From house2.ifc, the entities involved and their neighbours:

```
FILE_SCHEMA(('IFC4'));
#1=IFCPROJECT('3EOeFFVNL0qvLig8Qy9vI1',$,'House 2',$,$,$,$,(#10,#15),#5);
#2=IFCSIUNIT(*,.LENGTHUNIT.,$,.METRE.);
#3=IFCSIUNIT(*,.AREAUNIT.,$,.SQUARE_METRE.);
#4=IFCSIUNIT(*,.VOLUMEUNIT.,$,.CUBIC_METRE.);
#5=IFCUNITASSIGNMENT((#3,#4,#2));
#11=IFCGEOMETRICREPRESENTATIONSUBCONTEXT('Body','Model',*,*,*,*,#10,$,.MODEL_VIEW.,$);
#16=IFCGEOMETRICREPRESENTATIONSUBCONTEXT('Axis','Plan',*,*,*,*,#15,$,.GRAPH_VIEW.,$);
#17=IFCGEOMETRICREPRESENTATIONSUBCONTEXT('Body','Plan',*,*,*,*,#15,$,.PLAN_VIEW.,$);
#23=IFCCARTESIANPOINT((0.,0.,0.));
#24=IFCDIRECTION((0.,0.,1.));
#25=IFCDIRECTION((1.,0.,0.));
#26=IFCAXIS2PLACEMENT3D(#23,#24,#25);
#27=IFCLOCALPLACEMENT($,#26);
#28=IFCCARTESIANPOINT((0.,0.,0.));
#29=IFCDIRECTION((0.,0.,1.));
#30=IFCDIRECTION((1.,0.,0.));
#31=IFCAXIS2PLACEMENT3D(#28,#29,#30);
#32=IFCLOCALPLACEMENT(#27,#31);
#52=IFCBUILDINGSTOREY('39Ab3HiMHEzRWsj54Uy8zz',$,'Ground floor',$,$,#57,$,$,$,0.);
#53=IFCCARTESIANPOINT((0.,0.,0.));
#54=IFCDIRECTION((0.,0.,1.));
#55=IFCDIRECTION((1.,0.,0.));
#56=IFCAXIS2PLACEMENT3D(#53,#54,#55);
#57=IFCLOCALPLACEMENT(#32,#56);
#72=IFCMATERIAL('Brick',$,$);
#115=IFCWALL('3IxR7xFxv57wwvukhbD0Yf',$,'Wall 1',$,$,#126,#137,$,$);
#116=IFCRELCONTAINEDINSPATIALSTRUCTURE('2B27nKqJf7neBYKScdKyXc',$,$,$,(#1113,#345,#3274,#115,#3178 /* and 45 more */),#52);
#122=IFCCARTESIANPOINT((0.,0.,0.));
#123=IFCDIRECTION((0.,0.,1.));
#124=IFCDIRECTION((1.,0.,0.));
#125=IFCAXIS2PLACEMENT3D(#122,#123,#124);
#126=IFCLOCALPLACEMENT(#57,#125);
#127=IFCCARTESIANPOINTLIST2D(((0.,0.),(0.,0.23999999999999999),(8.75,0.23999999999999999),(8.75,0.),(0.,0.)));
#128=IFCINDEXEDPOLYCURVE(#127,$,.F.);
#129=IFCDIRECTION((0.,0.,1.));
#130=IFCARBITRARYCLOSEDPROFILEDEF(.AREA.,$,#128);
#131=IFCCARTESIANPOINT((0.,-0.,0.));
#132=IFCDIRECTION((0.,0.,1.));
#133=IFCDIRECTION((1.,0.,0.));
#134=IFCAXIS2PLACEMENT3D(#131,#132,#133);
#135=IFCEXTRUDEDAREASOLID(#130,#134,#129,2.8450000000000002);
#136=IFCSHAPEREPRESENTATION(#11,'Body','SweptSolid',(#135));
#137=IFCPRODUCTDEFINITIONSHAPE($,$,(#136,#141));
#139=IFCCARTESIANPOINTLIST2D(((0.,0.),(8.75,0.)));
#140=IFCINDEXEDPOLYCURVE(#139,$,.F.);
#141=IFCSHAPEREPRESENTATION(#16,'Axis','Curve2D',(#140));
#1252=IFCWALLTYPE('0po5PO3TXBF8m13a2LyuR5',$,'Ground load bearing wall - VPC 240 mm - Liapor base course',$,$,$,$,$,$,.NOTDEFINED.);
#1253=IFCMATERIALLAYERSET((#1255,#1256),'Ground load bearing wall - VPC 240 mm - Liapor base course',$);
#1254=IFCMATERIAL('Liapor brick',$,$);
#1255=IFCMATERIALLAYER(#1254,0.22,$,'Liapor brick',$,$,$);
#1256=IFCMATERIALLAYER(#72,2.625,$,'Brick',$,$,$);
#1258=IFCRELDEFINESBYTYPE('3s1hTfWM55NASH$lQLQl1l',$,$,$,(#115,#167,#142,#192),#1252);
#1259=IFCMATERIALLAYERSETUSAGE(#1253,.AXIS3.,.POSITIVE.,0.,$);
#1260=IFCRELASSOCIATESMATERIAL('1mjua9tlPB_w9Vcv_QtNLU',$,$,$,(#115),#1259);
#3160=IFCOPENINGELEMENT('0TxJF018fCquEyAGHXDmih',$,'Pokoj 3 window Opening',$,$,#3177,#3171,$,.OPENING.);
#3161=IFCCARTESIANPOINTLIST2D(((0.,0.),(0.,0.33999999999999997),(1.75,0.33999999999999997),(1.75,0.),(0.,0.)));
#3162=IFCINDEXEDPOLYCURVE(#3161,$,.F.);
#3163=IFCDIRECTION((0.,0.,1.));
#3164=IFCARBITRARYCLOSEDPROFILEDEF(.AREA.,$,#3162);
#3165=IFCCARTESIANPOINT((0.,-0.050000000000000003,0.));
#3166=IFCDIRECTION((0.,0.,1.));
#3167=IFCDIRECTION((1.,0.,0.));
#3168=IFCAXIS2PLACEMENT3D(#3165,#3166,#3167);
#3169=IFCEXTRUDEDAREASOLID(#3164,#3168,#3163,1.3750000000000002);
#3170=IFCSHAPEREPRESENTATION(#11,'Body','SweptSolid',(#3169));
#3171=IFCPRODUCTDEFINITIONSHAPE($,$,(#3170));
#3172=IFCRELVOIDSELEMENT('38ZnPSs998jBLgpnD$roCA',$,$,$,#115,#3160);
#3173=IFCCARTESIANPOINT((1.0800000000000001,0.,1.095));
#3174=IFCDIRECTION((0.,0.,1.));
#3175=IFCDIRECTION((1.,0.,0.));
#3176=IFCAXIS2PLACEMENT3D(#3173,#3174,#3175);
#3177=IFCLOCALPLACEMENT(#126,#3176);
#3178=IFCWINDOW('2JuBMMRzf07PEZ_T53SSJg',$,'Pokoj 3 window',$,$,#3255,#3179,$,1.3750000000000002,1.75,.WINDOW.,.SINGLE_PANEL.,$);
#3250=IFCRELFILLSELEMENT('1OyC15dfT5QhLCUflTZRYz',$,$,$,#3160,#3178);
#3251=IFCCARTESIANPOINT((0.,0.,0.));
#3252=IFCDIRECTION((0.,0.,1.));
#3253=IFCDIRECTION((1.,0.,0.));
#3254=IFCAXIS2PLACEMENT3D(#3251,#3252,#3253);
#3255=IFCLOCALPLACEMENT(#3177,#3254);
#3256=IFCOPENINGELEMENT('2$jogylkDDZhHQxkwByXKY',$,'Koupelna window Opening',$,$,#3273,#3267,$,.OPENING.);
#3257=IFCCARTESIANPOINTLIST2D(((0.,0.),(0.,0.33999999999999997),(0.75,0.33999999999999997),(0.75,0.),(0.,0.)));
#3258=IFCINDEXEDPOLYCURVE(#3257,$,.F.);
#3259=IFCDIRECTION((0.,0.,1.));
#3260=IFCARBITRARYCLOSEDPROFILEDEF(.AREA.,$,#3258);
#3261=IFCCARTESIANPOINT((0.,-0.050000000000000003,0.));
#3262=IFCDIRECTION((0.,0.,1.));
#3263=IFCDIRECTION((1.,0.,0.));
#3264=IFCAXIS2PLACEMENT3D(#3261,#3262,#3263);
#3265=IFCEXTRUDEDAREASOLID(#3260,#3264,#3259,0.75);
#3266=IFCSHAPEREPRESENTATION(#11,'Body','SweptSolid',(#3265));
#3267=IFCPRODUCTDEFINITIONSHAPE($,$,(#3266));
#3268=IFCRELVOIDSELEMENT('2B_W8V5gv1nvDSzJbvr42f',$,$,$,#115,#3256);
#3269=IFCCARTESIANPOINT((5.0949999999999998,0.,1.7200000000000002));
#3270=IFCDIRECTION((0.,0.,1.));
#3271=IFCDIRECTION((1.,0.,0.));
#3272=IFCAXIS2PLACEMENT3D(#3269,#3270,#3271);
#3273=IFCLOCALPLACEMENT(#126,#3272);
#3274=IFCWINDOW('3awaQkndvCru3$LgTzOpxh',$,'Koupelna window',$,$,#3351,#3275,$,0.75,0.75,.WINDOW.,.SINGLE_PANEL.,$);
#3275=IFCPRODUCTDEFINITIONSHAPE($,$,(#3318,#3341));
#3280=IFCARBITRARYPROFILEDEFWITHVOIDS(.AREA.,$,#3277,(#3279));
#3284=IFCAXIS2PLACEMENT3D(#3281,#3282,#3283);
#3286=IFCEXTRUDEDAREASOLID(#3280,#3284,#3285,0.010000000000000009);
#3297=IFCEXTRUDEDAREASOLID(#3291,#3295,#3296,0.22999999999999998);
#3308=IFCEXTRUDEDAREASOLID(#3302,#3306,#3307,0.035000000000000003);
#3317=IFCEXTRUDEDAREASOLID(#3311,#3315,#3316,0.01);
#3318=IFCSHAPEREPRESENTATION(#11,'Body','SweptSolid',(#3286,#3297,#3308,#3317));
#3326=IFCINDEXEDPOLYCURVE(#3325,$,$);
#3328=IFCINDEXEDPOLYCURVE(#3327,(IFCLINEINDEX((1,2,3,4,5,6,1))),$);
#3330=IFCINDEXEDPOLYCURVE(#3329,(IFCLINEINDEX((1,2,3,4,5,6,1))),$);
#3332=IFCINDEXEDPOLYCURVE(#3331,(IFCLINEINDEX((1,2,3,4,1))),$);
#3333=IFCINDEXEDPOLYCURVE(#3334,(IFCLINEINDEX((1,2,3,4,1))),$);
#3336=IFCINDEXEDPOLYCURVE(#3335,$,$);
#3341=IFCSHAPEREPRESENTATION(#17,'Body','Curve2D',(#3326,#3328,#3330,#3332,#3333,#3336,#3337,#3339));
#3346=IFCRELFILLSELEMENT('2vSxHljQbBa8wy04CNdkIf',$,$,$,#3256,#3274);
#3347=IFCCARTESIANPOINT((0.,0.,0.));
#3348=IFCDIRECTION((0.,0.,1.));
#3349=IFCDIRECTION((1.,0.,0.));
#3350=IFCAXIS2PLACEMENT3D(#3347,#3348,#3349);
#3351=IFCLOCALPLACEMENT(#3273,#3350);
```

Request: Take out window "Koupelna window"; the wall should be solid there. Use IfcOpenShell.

```python
import ifcopenshell
import ifcopenshell.api.feature
import ifcopenshell.api.root
import ifcopenshell.geom
import ifcopenshell.util.shape

model = ifcopenshell.open("house2.ifc")
settings = ifcopenshell.geom.settings()


def volume(element):
    """Net volume in cubic metres, openings subtracted."""
    shape = ifcopenshell.geom.create_shape(settings, element)
    return ifcopenshell.util.shape.get_volume(shape.geometry)


window = model.by_guid("3awaQkndvCru3$LgTzOpxh")
opening = window.FillsVoids[0].RelatingOpeningElement
wall = opening.VoidsElements[0].RelatingBuildingElement
before = volume(wall)

ifcopenshell.api.root.remove_product(model, product=window)
ifcopenshell.api.feature.remove_feature(model, feature=opening)

after = volume(wall)

print(f"wall volume {before:.3f} -> {after:.3f} m3")

model.write("house2_updated.ifc")
```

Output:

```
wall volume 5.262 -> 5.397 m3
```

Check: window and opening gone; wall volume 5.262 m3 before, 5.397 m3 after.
